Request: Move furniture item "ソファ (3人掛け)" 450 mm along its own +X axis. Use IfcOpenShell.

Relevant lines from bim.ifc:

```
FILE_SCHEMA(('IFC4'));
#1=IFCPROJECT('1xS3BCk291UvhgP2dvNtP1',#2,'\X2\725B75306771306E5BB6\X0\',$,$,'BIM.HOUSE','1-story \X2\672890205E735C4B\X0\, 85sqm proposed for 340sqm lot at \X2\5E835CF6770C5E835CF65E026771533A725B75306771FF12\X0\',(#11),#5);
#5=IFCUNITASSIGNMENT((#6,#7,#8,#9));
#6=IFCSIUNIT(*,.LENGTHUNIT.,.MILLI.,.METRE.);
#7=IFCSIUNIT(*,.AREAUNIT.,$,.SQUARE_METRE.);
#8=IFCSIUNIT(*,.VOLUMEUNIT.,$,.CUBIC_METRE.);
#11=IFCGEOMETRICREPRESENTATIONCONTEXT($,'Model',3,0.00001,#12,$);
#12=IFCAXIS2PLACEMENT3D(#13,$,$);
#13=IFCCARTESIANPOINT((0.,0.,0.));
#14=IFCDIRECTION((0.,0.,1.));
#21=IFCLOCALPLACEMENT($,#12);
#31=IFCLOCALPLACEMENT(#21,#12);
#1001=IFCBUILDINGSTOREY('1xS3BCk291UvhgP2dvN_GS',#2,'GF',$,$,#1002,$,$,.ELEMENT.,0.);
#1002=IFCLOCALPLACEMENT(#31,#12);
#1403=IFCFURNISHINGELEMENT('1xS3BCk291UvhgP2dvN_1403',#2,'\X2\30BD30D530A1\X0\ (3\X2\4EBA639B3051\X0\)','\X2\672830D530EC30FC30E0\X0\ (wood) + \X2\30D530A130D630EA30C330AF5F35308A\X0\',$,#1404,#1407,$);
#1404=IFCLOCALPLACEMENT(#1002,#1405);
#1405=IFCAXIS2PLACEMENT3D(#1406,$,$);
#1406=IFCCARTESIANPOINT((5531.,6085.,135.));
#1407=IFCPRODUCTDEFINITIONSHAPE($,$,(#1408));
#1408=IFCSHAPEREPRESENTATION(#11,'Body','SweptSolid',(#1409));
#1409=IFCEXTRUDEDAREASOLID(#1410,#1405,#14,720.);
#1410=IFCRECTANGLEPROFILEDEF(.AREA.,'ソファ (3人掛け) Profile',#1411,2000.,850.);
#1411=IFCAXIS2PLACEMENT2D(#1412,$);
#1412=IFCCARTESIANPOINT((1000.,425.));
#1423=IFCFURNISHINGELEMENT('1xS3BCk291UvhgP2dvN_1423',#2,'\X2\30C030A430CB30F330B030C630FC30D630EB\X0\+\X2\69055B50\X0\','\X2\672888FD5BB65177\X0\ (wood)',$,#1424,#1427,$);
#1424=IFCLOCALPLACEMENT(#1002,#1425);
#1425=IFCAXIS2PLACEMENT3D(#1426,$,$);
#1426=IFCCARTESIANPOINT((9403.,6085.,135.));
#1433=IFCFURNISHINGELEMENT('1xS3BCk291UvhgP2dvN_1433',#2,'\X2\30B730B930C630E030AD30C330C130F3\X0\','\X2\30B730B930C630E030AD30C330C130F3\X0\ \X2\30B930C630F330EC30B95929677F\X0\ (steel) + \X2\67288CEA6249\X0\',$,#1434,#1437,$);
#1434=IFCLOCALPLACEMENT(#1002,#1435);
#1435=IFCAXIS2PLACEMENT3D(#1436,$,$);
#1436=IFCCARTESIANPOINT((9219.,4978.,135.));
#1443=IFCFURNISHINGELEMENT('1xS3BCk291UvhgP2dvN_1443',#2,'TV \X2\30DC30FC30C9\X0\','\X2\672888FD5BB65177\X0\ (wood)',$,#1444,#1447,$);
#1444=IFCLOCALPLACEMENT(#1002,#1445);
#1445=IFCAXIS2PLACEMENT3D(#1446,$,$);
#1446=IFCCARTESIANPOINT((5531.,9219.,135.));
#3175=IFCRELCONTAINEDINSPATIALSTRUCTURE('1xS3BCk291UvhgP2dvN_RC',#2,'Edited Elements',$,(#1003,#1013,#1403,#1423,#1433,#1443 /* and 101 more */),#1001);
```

```python
import ifcopenshell
import ifcopenshell.api.geometry
import ifcopenshell.util.placement

model = ifcopenshell.open("bim.ifc")

item = model.by_guid("1xS3BCk291UvhgP2dvN_1403")
matrix = ifcopenshell.util.placement.get_local_placement(item.ObjectPlacement)
matrix[:3, 3] += matrix[:3, 0] * 450.0
ifcopenshell.api.geometry.edit_object_placement(model, product=item, matrix=matrix, is_si=False)

print(ifcopenshell.util.placement.get_local_placement(item.ObjectPlacement).round(3) + 0.0)

model.write("bim_v2.ifc")
```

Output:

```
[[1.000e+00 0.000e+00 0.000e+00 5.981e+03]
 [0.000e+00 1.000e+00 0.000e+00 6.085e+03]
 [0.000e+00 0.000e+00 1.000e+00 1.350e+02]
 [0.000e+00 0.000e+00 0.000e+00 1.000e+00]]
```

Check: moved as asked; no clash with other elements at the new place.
